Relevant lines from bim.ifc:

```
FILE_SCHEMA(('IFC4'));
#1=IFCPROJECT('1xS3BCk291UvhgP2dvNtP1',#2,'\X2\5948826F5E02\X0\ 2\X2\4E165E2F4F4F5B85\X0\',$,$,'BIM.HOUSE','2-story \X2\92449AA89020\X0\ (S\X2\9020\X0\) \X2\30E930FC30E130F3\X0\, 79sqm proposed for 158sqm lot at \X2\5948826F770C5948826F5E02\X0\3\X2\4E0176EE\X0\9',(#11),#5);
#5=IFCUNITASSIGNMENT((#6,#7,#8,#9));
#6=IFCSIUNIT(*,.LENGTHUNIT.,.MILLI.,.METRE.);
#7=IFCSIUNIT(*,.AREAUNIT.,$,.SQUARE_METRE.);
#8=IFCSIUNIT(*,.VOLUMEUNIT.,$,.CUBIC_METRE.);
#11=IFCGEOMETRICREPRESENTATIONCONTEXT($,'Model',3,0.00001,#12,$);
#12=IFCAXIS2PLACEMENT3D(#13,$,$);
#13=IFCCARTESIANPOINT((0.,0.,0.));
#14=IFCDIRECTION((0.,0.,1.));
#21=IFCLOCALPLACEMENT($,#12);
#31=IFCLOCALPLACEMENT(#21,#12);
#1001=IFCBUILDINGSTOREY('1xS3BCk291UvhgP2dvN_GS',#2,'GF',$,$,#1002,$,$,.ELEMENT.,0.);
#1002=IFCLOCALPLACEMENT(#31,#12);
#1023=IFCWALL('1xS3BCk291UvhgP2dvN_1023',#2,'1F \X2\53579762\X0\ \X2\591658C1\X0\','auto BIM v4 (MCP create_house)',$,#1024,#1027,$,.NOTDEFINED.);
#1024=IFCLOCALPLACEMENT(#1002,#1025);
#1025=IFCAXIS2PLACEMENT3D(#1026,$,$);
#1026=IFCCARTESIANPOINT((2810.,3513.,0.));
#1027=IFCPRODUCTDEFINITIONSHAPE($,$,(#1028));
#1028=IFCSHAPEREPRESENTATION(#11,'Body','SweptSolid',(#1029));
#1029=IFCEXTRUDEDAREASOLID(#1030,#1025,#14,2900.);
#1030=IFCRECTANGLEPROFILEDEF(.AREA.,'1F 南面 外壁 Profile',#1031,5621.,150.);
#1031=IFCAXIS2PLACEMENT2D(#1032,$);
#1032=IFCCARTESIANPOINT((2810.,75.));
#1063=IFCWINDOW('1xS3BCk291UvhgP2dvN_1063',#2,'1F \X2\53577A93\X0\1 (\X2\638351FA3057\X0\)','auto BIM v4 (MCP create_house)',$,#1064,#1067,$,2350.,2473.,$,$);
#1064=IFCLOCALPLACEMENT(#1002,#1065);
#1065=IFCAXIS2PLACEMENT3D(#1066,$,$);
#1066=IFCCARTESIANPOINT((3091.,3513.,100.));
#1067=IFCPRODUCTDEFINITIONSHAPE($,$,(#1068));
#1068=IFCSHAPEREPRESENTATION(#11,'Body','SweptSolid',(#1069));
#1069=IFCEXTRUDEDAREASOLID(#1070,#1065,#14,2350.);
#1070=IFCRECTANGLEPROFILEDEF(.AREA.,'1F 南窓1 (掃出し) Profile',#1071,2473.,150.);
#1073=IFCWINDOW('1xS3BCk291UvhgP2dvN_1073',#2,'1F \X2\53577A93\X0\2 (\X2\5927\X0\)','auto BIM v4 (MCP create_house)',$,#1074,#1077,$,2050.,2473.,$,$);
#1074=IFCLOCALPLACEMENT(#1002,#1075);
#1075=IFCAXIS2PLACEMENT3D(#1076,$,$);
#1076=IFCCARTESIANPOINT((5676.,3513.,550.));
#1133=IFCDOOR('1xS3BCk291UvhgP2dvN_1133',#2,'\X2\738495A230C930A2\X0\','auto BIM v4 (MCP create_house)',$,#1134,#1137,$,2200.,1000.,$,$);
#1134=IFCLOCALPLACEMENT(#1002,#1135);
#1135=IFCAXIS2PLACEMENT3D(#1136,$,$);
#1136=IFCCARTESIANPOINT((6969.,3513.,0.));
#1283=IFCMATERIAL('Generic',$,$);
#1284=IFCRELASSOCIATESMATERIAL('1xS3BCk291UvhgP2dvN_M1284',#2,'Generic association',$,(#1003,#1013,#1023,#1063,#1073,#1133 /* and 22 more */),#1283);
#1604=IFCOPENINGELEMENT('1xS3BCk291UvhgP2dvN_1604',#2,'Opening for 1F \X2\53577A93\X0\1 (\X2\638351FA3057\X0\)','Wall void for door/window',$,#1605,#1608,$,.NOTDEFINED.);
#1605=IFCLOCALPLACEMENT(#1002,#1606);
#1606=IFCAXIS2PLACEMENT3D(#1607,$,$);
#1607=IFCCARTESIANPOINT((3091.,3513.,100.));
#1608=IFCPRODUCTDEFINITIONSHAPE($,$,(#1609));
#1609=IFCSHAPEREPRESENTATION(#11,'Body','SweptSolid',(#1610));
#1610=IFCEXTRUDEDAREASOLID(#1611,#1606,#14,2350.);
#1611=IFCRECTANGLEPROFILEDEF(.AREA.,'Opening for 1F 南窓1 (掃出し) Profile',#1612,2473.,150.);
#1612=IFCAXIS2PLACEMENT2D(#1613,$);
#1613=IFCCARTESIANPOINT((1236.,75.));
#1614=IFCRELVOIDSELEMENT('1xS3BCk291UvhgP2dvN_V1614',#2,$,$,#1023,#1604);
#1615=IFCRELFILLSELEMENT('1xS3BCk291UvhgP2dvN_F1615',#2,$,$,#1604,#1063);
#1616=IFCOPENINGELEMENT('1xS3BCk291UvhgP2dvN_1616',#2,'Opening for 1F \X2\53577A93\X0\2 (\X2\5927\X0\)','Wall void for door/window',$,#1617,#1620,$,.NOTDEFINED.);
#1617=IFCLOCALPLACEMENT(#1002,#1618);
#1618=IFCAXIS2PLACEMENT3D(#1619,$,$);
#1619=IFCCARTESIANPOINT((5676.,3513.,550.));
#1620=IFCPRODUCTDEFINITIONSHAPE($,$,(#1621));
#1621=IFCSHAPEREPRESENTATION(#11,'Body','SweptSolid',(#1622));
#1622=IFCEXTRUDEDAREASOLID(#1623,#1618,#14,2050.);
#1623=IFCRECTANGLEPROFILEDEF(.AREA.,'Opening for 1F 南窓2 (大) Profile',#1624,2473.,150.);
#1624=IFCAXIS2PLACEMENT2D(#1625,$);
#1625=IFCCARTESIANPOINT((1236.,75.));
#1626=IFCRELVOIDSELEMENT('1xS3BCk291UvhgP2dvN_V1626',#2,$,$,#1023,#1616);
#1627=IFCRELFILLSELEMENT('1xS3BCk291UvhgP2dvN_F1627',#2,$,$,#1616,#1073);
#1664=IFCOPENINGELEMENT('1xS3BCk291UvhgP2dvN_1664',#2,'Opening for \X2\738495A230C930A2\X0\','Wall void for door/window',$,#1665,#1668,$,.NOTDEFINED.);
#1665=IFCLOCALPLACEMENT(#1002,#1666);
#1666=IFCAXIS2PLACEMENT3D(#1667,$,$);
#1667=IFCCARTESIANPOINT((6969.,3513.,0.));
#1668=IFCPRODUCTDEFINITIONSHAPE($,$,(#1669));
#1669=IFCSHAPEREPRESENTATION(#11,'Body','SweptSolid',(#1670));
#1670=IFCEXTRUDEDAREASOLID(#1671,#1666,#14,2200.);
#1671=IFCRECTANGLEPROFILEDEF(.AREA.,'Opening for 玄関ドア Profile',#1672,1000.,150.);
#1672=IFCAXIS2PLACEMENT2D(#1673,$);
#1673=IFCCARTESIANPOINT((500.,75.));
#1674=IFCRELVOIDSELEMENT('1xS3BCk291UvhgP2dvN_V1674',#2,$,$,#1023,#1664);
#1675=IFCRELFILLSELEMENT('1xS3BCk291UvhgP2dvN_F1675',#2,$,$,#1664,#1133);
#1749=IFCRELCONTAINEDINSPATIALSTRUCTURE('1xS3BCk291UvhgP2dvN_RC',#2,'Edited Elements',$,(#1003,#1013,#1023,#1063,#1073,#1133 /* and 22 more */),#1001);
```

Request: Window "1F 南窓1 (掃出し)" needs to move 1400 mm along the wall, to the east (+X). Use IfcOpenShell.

```python
import ifcopenshell
import ifcopenshell.api.geometry
import ifcopenshell.util.placement
import ifcopenshell.util.unit

model = ifcopenshell.open("bim.ifc")
unit_scale = ifcopenshell.util.unit.calculate_unit_scale(model)

window = model.by_guid("1xS3BCk291UvhgP2dvN_1063")
opening = window.FillsVoids[0].RelatingOpeningElement
wall = opening.VoidsElements[0].RelatingBuildingElement

wall_matrix = ifcopenshell.util.placement.get_local_placement(wall.ObjectPlacement)
shift = wall_matrix[:3, 0] * 1.4 / unit_scale
before = ifcopenshell.util.placement.get_local_placement(window.ObjectPlacement)[:3, 3].copy()

# The window is not placed relative to its opening, so move both.
for product in (opening, window):
    matrix = ifcopenshell.util.placement.get_local_placement(product.ObjectPlacement)
    matrix[:3, 3] += shift
    ifcopenshell.api.geometry.edit_object_placement(model, product=product, matrix=matrix, is_si=False)

after = ifcopenshell.util.placement.get_local_placement(window.ObjectPlacement)[:3, 3]
print("window moved by", (after - before).round(3) + 0.0)

model.write("bim_updated.ifc")
```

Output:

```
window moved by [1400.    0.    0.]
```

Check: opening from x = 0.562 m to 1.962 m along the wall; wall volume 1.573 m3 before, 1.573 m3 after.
